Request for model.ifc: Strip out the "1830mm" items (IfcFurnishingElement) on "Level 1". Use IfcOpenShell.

First a look at what the model holds.

```python
import ifcopenshell
import ifcopenshell.util.element

model = ifcopenshell.open("model.ifc")
print(model.schema)
storey = next(s for s in model.by_type("IfcBuildingStorey") if s.Name == "Level 1")
furniture = [e for e in ifcopenshell.util.element.get_decomposition(storey) if e.is_a("IfcFurnishingElement")]
seen = {}
for e in furniture:
    element_type = ifcopenshell.util.element.get_type(e)
    name = element_type.Name if element_type not in (None, e) else None
    seen[name] = seen.get(name, 0) + 1
for name, count in sorted(seen.items(), key=str):
    print(count, "x", name)
```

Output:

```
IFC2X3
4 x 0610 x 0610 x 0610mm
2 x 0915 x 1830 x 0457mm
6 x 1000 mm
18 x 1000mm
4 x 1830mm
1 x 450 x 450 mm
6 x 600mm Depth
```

```python
import ifcopenshell
import ifcopenshell.api.root
import ifcopenshell.util.element

model = ifcopenshell.open("model.ifc")

storey = next(s for s in model.by_type("IfcBuildingStorey") if s.Name == "Level 1")
furniture = [e for e in ifcopenshell.util.element.get_decomposition(storey) if e.is_a("IfcFurnishingElement")]
targets = [e for e in furniture if (t := ifcopenshell.util.element.get_type(e)) not in (None, e) and t.Name == "1830mm"]

for e in targets:
    ifcopenshell.api.root.remove_product(model, product=e)
print(len(targets), "removed")

model.write("model_v2.ifc")
```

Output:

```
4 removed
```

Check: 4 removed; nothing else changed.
